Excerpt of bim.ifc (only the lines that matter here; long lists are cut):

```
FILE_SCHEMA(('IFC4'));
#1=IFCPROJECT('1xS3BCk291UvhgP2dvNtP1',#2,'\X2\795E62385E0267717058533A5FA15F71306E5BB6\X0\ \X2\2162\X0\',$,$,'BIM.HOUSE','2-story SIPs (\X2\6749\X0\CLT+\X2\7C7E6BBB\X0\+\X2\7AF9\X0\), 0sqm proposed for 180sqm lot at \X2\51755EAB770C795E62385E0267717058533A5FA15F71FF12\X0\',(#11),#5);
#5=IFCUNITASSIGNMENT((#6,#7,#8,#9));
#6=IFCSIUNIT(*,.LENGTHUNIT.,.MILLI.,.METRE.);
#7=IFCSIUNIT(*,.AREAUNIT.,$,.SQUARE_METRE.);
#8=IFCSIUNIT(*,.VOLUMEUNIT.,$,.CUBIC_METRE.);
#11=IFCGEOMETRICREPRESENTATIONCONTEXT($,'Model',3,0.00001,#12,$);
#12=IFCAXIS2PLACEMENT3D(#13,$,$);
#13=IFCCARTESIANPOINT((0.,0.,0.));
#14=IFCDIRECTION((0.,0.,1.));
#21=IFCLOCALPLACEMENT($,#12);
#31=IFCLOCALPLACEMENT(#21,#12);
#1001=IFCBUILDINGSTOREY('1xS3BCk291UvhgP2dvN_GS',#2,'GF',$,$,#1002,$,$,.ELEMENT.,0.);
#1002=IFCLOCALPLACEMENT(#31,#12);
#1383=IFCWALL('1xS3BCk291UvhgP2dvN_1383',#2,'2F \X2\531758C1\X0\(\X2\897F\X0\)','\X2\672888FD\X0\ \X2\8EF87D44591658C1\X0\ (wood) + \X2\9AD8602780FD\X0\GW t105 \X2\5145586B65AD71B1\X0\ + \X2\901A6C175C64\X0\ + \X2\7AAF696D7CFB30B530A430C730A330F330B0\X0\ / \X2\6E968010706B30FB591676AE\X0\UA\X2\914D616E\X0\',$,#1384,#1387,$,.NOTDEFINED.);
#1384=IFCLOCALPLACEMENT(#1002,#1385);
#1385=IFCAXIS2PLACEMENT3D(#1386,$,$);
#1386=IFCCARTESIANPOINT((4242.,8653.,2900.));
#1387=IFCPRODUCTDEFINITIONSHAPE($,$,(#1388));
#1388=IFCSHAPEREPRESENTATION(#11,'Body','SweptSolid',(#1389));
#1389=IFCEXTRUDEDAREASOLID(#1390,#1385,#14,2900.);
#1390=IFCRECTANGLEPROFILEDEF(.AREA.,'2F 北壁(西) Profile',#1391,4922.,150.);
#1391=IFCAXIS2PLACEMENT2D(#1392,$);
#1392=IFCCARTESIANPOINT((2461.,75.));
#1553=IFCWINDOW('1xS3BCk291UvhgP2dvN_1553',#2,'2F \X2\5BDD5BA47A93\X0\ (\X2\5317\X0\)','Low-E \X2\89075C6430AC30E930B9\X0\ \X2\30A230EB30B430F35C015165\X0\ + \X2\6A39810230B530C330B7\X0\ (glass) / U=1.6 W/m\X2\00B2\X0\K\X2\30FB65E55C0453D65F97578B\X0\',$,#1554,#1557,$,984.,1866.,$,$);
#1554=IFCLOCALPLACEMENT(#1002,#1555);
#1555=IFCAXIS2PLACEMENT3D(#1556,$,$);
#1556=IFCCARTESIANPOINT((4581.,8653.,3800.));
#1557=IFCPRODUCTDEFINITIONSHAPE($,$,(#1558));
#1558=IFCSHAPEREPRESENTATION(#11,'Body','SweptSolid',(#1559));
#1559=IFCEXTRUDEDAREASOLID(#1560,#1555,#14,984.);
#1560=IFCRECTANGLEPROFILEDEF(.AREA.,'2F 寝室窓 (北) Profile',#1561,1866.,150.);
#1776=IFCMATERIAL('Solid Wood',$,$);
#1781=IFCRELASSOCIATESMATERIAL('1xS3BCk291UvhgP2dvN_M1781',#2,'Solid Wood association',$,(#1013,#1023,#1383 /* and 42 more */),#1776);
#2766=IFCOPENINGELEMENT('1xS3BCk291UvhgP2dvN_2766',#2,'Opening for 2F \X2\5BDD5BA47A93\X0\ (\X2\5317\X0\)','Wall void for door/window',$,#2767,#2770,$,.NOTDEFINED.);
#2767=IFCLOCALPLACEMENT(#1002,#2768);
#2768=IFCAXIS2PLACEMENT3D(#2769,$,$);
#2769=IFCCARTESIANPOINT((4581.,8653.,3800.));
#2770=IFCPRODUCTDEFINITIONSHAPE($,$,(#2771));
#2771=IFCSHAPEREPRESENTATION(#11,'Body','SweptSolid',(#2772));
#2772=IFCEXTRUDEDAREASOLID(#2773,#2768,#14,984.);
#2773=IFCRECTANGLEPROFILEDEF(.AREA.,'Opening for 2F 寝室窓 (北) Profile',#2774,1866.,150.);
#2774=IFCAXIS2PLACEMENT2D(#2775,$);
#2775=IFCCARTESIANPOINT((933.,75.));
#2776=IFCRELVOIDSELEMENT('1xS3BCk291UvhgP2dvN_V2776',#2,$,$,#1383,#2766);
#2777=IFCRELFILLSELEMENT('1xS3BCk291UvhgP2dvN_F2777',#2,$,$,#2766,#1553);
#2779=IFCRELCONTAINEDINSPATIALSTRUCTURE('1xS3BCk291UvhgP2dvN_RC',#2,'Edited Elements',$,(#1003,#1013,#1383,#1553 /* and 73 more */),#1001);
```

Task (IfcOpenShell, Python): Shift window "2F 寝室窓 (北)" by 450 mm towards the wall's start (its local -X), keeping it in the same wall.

```python
import ifcopenshell
import ifcopenshell.api.geometry
import ifcopenshell.util.placement
import ifcopenshell.util.unit

model = ifcopenshell.open("bim.ifc")
unit_scale = ifcopenshell.util.unit.calculate_unit_scale(model)

window = model.by_guid("1xS3BCk291UvhgP2dvN_1553")
opening = window.FillsVoids[0].RelatingOpeningElement
wall = opening.VoidsElements[0].RelatingBuildingElement

wall_matrix = ifcopenshell.util.placement.get_local_placement(wall.ObjectPlacement)
shift = wall_matrix[:3, 0] * -0.45 / unit_scale
before = ifcopenshell.util.placement.get_local_placement(window.ObjectPlacement)[:3, 3].copy()

# The window is not placed relative to its opening, so move both.
for product in (opening, window):
    matrix = ifcopenshell.util.placement.get_local_placement(product.ObjectPlacement)
    matrix[:3, 3] += shift
    ifcopenshell.api.geometry.edit_object_placement(model, product=product, matrix=matrix, is_si=False)

after = ifcopenshell.util.placement.get_local_placement(window.ObjectPlacement)[:3, 3]
print("window moved by", (after - before).round(3) + 0.0)

model.write("bim_rev.ifc")
```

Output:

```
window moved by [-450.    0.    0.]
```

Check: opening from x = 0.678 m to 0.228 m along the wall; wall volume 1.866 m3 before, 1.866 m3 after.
